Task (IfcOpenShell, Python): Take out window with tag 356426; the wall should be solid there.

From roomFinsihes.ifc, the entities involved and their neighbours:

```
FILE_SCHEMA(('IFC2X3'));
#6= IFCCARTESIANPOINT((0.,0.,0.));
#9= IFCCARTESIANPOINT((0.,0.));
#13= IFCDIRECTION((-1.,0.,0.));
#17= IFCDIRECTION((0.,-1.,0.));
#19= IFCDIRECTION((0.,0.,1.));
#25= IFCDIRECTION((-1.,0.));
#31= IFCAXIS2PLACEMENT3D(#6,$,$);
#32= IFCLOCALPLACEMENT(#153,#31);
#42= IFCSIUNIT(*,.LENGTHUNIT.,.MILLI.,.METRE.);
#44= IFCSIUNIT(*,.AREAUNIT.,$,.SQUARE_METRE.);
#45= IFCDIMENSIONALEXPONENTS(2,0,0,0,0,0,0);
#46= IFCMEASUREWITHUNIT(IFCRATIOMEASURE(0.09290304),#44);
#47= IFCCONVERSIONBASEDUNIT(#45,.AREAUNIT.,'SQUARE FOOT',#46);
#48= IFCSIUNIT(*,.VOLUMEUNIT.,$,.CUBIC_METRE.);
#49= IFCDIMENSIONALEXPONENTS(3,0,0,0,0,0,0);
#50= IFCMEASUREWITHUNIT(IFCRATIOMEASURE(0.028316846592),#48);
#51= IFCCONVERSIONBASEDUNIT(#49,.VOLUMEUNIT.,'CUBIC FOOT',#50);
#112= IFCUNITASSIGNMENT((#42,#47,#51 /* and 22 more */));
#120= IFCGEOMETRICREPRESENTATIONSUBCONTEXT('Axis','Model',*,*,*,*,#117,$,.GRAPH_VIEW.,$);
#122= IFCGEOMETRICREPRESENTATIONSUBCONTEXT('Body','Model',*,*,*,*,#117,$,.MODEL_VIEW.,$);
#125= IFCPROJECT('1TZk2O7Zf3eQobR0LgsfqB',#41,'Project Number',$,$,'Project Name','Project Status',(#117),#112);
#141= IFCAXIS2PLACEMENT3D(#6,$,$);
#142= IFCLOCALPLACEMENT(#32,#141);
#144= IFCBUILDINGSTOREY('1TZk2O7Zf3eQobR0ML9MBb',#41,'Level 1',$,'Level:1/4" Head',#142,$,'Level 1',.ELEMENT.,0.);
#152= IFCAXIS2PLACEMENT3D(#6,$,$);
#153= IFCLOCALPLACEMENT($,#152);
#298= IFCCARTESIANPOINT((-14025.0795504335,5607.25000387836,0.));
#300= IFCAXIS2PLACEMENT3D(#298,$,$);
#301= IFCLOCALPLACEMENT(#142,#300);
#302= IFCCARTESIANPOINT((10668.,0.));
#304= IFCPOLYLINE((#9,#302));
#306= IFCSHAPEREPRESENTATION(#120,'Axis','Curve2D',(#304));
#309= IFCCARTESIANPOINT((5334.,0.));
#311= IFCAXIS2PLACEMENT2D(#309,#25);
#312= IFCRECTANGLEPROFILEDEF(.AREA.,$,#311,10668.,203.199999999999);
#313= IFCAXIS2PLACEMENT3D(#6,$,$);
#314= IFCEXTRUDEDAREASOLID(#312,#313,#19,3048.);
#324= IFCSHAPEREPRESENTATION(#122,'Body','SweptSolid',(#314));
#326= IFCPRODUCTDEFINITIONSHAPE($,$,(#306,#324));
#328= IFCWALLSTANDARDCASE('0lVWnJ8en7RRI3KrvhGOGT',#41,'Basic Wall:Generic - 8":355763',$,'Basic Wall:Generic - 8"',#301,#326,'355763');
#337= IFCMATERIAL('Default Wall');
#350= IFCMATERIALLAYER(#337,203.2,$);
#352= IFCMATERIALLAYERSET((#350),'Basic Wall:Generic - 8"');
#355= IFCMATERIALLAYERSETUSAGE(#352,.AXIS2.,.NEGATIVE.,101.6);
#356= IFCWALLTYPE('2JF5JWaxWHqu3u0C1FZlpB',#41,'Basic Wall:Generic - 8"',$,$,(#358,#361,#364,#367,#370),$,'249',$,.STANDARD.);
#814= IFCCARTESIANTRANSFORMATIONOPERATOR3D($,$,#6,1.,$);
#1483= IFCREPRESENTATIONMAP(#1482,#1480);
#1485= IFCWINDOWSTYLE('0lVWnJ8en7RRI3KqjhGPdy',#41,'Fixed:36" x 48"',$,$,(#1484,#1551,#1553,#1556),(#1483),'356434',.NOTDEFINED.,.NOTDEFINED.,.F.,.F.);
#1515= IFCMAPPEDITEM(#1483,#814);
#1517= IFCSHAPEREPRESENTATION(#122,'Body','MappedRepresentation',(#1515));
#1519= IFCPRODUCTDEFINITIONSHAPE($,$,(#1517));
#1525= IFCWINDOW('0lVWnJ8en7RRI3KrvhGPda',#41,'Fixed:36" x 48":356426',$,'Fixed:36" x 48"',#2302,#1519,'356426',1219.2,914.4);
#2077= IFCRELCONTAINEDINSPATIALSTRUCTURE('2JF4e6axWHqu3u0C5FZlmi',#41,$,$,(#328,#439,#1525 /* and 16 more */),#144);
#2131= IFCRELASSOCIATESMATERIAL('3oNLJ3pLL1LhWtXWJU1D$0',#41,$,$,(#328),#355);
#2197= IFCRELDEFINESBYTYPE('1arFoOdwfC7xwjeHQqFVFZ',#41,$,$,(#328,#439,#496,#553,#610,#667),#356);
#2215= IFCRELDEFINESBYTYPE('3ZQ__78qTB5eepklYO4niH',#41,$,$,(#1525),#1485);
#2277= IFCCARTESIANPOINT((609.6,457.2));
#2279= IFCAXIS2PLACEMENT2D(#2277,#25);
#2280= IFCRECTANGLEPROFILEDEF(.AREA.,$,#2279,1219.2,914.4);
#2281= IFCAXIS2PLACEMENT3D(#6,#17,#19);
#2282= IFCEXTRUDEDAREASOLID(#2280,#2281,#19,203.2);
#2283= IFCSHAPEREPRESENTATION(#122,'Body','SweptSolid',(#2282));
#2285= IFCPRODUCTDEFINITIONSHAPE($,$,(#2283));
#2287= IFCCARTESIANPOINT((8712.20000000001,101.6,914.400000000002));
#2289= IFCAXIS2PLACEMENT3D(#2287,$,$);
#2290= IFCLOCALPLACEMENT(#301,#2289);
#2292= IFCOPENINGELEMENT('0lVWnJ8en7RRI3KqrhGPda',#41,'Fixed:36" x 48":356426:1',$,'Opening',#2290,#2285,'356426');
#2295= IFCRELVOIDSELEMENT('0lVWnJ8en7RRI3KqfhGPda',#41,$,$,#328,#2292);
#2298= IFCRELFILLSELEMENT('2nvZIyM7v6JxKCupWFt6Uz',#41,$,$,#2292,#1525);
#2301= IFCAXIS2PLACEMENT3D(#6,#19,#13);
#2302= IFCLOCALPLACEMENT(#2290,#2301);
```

```python
import ifcopenshell
import ifcopenshell.api.feature
import ifcopenshell.api.root
import ifcopenshell.geom
import ifcopenshell.util.shape

model = ifcopenshell.open("roomFinsihes.ifc")
settings = ifcopenshell.geom.settings()


def volume(element):
    """Net volume in cubic metres, openings subtracted."""
    shape = ifcopenshell.geom.create_shape(settings, element)
    return ifcopenshell.util.shape.get_volume(shape.geometry)


window = model.by_guid("0lVWnJ8en7RRI3KrvhGPda")
opening = window.FillsVoids[0].RelatingOpeningElement
wall = opening.VoidsElements[0].RelatingBuildingElement
before = volume(wall)

ifcopenshell.api.root.remove_product(model, product=window)
ifcopenshell.api.feature.remove_feature(model, feature=opening)

after = volume(wall)

print(f"wall volume {before:.3f} -> {after:.3f} m3")

model.write("roomFinsihes_updated.ifc")
```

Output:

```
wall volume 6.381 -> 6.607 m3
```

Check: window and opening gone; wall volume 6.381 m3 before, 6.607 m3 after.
